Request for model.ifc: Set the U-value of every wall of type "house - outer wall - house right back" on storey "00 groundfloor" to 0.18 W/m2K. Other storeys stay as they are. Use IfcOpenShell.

First a look at what the model holds.

```python
import ifcopenshell
import ifcopenshell.util.element

model = ifcopenshell.open("model.ifc")
print(model.schema)
storey = next(s for s in model.by_type("IfcBuildingStorey") if s.Name == "00 groundfloor")
walls = [e for e in ifcopenshell.util.element.get_decomposition(storey) if e.is_a("IfcWall")]
seen = {}
for e in walls:
    element_type = ifcopenshell.util.element.get_type(e)
    key = (element_type.Name if element_type != e and element_type else None, ifcopenshell.util.element.get_pset(e, "Pset_WallCommon", "ThermalTransmittance"))
    seen[key] = seen.get(key, 0) + 1
for (name, value), count in sorted(seen.items(), key=str):
    print(count, "x", name, "|", value)
```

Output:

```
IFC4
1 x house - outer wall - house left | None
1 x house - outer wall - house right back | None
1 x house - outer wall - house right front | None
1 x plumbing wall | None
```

```python
import ifcopenshell
import ifcopenshell.api.pset
import ifcopenshell.util.element

model = ifcopenshell.open("model.ifc")

storey = next(s for s in model.by_type("IfcBuildingStorey") if s.Name == "00 groundfloor")
walls = [e for e in ifcopenshell.util.element.get_decomposition(storey) if e.is_a("IfcWall")]

count = 0
for e in walls:
    element_type = ifcopenshell.util.element.get_type(e)
    if element_type in (None, e) or element_type.Name != "house - outer wall - house right back":
        continue
    # add_pset returns the element's existing set when there is one.
    pset = ifcopenshell.api.pset.add_pset(model, product=e, name="Pset_WallCommon")
    ifcopenshell.api.pset.edit_pset(model, pset=pset, properties={"ThermalTransmittance": 0.18})
    count += 1

print(count, "walls updated")

model.write("model_edited.ifc")
```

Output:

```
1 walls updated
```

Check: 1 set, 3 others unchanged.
